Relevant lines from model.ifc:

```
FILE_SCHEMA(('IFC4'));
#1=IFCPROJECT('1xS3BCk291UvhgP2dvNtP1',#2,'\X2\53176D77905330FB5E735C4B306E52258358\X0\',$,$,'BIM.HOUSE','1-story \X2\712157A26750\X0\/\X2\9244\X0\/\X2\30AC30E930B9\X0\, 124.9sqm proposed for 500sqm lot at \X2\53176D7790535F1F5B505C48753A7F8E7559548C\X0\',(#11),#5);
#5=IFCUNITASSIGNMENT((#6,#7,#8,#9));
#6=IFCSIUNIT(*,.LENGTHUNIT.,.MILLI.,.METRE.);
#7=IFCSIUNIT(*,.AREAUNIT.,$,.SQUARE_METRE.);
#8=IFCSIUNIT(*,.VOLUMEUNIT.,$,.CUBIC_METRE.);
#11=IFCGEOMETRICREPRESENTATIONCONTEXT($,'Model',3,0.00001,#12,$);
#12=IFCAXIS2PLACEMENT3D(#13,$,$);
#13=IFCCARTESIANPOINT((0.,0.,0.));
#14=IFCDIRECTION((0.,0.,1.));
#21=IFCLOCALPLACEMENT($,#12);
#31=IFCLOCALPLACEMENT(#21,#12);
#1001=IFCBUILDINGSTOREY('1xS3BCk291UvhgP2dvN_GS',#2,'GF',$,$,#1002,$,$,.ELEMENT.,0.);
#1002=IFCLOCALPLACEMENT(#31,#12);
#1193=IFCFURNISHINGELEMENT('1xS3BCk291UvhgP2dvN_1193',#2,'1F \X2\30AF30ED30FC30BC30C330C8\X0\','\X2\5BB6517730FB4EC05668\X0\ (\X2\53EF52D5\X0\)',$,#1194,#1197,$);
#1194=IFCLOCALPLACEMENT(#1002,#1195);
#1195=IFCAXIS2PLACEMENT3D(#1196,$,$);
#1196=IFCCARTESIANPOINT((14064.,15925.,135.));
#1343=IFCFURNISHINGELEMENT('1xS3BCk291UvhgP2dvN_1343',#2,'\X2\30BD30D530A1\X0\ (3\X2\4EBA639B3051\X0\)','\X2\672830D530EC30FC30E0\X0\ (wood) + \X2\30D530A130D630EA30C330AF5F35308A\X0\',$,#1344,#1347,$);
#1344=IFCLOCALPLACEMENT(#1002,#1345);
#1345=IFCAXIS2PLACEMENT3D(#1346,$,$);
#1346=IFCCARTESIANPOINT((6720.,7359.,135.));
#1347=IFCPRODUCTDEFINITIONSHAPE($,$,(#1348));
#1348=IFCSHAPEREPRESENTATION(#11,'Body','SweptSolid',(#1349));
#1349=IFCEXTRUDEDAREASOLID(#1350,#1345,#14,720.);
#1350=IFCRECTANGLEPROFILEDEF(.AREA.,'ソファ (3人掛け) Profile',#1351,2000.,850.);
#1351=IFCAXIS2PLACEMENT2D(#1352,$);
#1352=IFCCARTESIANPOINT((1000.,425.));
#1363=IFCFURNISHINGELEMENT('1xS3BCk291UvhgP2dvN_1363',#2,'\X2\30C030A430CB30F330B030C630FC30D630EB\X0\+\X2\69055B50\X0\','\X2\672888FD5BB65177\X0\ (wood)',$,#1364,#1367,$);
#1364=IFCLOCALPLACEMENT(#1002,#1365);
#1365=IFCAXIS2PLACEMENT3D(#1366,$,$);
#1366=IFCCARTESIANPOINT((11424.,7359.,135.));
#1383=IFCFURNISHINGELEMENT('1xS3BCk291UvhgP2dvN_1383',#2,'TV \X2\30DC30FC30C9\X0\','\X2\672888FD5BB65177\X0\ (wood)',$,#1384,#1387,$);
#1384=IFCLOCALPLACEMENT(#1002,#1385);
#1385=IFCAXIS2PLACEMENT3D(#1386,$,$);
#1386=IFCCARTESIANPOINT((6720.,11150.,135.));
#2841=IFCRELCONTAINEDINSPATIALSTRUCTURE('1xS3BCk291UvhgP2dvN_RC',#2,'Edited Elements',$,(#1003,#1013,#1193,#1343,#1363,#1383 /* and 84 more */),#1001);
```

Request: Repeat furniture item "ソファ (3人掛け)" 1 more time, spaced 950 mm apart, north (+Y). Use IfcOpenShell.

```python
import numpy as np
import ifcopenshell
import ifcopenshell.api.geometry
import ifcopenshell.api.root
import ifcopenshell.util.element
import ifcopenshell.util.placement
import ifcopenshell.util.unit

model = ifcopenshell.open("model.ifc")
unit_scale = ifcopenshell.util.unit.calculate_unit_scale(model)


def reuse_history(source, copy):
    """copy_class also copies each property set's owner history, people and application; keep the originals."""
    for rel in copy.IsDefinedBy:
        if rel.is_a("IfcRelDefinesByProperties") and (history := rel.RelatingPropertyDefinition.OwnerHistory):
            rel.RelatingPropertyDefinition.OwnerHistory = source.OwnerHistory
            ifcopenshell.util.element.remove_deep2(model, history)


source = model.by_guid("1xS3BCk291UvhgP2dvN_1343")
base = ifcopenshell.util.placement.get_local_placement(source.ObjectPlacement)
step = np.array([0.0, 1.0, 0.0]) * 0.95 / unit_scale

for i in range(1, 2):
    copy = ifcopenshell.api.root.copy_class(model, product=source)
    copy.Representation = ifcopenshell.util.element.copy_deep(
        model, source.Representation, exclude=["IfcGeometricRepresentationContext", "IfcRepresentationMap"]
    )
    reuse_history(source, copy)
    matrix = base.copy()
    matrix[:3, 3] += i * step
    print("added at", matrix[:3, 3].round(3) + 0.0)
    ifcopenshell.api.geometry.edit_object_placement(model, product=copy, matrix=matrix, is_si=False)

model.write("model_edited.ifc")
```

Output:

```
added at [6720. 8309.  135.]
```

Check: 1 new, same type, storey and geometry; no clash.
